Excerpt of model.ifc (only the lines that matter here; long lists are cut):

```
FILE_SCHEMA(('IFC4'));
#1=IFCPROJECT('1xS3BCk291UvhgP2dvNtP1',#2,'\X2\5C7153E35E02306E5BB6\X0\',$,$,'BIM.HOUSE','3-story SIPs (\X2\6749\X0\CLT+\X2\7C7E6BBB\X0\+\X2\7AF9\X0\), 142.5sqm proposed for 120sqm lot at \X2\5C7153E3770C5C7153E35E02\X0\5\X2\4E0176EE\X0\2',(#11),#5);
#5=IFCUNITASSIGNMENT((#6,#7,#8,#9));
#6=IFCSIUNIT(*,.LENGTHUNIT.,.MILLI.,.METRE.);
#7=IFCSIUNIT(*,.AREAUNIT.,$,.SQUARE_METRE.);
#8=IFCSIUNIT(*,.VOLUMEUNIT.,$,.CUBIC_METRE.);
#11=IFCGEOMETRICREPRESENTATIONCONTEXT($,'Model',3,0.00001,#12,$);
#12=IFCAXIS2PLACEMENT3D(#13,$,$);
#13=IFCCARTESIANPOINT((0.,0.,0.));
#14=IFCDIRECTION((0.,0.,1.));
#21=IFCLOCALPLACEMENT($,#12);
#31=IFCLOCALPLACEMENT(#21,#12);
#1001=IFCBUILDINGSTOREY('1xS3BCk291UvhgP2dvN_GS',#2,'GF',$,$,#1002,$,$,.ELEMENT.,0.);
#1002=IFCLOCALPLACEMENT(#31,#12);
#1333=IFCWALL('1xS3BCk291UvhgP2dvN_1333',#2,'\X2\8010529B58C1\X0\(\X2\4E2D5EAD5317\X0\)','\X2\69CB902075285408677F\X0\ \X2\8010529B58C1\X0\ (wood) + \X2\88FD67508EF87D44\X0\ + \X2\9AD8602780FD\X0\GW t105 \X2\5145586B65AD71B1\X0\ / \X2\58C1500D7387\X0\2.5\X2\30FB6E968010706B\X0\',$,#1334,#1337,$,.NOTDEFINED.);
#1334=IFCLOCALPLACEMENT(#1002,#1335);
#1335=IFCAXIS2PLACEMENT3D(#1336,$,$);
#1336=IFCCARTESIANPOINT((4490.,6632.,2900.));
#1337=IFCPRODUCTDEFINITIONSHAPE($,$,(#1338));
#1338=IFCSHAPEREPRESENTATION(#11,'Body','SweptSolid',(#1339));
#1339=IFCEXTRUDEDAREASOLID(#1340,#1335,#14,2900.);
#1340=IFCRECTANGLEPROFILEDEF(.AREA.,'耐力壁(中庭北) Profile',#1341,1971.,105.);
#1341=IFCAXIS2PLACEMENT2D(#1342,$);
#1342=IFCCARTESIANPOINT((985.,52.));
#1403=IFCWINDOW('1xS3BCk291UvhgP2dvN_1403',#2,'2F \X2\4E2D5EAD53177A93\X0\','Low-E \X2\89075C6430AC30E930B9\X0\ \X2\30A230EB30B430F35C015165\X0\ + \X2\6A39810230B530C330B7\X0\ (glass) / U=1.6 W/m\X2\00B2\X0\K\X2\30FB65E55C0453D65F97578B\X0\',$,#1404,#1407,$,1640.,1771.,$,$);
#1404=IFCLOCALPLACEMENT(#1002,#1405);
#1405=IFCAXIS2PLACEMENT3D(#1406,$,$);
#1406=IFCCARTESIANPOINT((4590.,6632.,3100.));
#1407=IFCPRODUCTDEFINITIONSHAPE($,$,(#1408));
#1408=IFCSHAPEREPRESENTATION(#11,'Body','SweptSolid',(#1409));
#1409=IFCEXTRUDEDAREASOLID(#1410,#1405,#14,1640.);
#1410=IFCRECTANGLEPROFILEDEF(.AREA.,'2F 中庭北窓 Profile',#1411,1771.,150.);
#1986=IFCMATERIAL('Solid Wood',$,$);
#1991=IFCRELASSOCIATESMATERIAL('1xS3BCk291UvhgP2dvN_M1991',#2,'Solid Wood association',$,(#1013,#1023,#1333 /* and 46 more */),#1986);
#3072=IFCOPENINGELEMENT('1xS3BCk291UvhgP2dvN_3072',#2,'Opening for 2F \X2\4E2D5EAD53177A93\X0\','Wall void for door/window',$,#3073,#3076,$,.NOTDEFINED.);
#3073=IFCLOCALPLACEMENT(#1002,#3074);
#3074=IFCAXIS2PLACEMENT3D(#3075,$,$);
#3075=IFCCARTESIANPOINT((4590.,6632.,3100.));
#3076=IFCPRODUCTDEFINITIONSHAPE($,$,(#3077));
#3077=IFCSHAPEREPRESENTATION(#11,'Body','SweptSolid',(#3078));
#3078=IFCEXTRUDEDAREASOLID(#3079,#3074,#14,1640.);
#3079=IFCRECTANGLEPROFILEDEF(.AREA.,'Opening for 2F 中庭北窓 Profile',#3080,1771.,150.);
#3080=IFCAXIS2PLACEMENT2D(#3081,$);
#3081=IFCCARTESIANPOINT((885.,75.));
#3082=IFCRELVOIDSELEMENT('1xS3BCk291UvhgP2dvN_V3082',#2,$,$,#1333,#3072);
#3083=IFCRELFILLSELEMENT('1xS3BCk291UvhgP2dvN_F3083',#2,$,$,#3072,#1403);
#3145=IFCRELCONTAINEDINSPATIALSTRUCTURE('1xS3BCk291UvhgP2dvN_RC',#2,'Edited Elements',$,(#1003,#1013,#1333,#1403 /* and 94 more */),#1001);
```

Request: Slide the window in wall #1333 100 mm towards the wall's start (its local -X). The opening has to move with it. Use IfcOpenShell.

```python
import ifcopenshell
import ifcopenshell.api.geometry
import ifcopenshell.util.placement
import ifcopenshell.util.unit

model = ifcopenshell.open("model.ifc")
unit_scale = ifcopenshell.util.unit.calculate_unit_scale(model)

window = model.by_guid("1xS3BCk291UvhgP2dvN_1403")
opening = window.FillsVoids[0].RelatingOpeningElement
wall = opening.VoidsElements[0].RelatingBuildingElement

wall_matrix = ifcopenshell.util.placement.get_local_placement(wall.ObjectPlacement)
shift = wall_matrix[:3, 0] * -0.1 / unit_scale
before = ifcopenshell.util.placement.get_local_placement(window.ObjectPlacement)[:3, 3].copy()

# The window is not placed relative to its opening, so move both.
for product in (opening, window):
    matrix = ifcopenshell.util.placement.get_local_placement(product.ObjectPlacement)
    matrix[:3, 3] += shift
    ifcopenshell.api.geometry.edit_object_placement(model, product=product, matrix=matrix, is_si=False)

after = ifcopenshell.util.placement.get_local_placement(window.ObjectPlacement)[:3, 3]
print("window moved by", (after - before).round(3) + 0.0)

model.write("model_edited.ifc")
```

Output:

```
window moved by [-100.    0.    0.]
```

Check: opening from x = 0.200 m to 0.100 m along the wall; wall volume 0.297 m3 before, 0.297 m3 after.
